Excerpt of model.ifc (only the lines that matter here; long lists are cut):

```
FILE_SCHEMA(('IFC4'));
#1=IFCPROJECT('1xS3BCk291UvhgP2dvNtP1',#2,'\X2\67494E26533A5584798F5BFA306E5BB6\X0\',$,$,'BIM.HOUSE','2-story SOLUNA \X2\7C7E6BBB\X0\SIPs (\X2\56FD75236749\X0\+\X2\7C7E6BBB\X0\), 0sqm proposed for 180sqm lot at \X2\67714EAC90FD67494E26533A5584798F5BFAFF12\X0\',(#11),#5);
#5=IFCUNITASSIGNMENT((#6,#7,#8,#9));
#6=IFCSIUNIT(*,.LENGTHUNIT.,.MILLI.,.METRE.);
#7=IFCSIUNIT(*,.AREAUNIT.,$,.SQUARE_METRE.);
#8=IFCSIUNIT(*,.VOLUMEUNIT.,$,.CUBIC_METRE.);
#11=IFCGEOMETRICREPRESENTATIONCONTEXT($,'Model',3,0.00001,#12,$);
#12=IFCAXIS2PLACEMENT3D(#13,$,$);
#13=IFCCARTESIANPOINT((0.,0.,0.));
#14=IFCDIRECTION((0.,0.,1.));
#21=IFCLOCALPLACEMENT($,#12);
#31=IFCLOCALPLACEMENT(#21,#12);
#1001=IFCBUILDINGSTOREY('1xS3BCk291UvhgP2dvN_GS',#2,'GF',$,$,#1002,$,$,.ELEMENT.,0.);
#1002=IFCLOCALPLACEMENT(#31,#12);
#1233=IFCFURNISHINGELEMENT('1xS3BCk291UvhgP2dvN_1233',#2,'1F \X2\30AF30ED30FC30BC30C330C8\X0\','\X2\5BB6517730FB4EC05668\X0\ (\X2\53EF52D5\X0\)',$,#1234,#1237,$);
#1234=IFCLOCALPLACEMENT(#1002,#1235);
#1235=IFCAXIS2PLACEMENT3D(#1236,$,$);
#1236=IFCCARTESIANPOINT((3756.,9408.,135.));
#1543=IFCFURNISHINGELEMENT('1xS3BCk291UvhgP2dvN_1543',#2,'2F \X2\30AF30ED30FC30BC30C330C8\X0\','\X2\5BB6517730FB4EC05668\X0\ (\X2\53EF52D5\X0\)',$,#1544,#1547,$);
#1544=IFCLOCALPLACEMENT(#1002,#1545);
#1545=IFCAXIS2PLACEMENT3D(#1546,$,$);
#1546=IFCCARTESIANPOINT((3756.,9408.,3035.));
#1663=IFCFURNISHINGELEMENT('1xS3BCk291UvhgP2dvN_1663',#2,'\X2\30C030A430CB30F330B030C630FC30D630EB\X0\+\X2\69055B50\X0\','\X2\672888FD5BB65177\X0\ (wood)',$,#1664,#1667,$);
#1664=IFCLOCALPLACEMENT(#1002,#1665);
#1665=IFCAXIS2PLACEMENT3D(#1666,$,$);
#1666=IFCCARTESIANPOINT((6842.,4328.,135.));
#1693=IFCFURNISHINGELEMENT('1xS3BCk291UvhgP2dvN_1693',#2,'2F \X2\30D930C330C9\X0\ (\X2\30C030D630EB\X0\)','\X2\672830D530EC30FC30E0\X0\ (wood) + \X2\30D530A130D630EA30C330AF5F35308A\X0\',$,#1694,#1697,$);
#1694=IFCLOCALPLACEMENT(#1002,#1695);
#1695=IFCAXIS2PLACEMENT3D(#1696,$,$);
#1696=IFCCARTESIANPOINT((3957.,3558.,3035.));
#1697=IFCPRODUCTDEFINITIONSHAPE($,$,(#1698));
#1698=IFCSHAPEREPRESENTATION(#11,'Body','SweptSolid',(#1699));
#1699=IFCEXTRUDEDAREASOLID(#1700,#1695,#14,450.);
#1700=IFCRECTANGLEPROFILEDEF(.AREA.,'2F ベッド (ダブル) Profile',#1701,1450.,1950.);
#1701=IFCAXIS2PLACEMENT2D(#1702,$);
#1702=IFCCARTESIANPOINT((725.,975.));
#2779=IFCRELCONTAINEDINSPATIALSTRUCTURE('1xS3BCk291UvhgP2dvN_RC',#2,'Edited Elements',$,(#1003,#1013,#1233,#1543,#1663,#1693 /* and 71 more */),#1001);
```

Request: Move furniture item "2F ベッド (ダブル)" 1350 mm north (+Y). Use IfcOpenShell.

```python
import ifcopenshell
import ifcopenshell.api.geometry
import ifcopenshell.util.placement
import ifcopenshell.util.unit

model = ifcopenshell.open("model.ifc")
unit_scale = ifcopenshell.util.unit.calculate_unit_scale(model)

item = model.by_id(1693)
matrix = ifcopenshell.util.placement.get_local_placement(item.ObjectPlacement)
matrix[1, 3] += 1.35 / unit_scale
ifcopenshell.api.geometry.edit_object_placement(model, product=item, matrix=matrix, is_si=False)

print(ifcopenshell.util.placement.get_local_placement(item.ObjectPlacement).round(3) + 0.0)

model.write("model_v2.ifc")
```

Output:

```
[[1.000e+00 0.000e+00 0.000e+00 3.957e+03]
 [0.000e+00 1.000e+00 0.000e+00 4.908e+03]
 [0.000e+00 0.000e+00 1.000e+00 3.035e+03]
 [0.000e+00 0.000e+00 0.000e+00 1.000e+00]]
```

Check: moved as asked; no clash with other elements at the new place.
